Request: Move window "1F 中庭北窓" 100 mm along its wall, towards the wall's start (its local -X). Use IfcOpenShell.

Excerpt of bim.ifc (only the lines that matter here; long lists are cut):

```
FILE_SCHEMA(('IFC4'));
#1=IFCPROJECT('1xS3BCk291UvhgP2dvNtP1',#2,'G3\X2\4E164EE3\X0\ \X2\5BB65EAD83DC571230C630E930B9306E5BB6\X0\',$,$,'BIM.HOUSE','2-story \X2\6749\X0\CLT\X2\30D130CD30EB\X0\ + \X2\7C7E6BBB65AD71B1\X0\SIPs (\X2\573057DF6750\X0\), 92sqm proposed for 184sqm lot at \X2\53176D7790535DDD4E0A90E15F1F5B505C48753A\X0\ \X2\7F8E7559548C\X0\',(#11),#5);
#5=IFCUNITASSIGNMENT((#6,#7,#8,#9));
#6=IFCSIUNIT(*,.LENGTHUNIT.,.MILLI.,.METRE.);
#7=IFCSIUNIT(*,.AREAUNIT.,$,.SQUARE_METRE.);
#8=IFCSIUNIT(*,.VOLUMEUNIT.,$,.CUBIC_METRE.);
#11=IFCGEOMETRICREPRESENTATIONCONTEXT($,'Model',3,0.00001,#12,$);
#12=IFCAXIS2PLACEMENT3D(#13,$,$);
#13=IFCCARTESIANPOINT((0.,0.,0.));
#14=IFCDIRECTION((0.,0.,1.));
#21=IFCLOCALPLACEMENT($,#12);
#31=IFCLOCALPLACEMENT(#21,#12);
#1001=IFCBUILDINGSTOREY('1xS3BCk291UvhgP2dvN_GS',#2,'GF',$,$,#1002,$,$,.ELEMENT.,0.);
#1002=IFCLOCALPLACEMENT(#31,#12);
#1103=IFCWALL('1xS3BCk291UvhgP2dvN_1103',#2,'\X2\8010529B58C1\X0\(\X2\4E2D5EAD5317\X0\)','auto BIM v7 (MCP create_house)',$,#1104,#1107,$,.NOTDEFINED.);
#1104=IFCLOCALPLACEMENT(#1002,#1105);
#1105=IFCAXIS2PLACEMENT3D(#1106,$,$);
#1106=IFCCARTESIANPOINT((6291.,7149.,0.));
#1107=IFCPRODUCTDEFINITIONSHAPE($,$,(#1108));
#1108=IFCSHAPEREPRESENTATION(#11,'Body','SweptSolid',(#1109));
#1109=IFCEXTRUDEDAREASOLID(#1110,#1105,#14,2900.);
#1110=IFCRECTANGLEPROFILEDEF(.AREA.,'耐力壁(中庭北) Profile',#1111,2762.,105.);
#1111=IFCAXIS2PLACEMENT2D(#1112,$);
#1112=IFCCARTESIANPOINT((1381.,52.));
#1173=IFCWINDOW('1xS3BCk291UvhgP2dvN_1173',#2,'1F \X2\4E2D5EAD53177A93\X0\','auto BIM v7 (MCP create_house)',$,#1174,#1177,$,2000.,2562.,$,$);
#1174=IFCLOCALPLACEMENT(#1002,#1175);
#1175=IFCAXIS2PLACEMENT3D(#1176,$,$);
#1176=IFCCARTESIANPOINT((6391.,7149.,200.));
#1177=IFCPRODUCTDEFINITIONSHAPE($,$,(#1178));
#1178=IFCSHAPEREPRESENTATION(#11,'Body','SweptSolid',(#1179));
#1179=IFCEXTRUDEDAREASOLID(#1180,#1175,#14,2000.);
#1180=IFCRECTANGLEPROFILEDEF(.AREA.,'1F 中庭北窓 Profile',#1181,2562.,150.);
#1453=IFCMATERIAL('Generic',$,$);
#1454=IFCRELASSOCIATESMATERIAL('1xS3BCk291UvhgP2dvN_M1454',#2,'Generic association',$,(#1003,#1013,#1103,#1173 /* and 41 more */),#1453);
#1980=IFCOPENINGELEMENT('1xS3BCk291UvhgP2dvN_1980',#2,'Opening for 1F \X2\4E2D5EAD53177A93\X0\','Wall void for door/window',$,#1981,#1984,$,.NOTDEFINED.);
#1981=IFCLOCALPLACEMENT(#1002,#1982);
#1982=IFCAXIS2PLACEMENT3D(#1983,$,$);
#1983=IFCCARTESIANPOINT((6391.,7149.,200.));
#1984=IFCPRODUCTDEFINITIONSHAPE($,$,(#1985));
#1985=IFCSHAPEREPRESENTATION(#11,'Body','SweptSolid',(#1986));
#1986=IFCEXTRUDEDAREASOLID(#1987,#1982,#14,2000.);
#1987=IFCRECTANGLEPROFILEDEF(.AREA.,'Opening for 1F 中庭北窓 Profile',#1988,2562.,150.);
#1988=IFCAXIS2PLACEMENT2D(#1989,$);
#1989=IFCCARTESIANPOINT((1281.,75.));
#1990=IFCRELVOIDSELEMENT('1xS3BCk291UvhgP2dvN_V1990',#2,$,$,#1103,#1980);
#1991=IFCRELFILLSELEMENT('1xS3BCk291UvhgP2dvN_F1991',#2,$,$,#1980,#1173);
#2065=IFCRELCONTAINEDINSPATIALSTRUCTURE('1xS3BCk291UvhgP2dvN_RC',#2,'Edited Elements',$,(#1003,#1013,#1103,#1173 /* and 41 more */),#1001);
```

```python
import ifcopenshell
import ifcopenshell.api.geometry
import ifcopenshell.util.placement
import ifcopenshell.util.unit

model = ifcopenshell.open("bim.ifc")
unit_scale = ifcopenshell.util.unit.calculate_unit_scale(model)

window = model.by_guid("1xS3BCk291UvhgP2dvN_1173")
opening = window.FillsVoids[0].RelatingOpeningElement
wall = opening.VoidsElements[0].RelatingBuildingElement

wall_matrix = ifcopenshell.util.placement.get_local_placement(wall.ObjectPlacement)
shift = wall_matrix[:3, 0] * -0.1 / unit_scale
before = ifcopenshell.util.placement.get_local_placement(window.ObjectPlacement)[:3, 3].copy()

# The window is not placed relative to its opening, so move both.
for product in (opening, window):
    matrix = ifcopenshell.util.placement.get_local_placement(product.ObjectPlacement)
    matrix[:3, 3] += shift
    ifcopenshell.api.geometry.edit_object_placement(model, product=product, matrix=matrix, is_si=False)

after = ifcopenshell.util.placement.get_local_placement(window.ObjectPlacement)[:3, 3]
print("window moved by", (after - before).round(3) + 0.0)

model.write("bim_rev.ifc")
```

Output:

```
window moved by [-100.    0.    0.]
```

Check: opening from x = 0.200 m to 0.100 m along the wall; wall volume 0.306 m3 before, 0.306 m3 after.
